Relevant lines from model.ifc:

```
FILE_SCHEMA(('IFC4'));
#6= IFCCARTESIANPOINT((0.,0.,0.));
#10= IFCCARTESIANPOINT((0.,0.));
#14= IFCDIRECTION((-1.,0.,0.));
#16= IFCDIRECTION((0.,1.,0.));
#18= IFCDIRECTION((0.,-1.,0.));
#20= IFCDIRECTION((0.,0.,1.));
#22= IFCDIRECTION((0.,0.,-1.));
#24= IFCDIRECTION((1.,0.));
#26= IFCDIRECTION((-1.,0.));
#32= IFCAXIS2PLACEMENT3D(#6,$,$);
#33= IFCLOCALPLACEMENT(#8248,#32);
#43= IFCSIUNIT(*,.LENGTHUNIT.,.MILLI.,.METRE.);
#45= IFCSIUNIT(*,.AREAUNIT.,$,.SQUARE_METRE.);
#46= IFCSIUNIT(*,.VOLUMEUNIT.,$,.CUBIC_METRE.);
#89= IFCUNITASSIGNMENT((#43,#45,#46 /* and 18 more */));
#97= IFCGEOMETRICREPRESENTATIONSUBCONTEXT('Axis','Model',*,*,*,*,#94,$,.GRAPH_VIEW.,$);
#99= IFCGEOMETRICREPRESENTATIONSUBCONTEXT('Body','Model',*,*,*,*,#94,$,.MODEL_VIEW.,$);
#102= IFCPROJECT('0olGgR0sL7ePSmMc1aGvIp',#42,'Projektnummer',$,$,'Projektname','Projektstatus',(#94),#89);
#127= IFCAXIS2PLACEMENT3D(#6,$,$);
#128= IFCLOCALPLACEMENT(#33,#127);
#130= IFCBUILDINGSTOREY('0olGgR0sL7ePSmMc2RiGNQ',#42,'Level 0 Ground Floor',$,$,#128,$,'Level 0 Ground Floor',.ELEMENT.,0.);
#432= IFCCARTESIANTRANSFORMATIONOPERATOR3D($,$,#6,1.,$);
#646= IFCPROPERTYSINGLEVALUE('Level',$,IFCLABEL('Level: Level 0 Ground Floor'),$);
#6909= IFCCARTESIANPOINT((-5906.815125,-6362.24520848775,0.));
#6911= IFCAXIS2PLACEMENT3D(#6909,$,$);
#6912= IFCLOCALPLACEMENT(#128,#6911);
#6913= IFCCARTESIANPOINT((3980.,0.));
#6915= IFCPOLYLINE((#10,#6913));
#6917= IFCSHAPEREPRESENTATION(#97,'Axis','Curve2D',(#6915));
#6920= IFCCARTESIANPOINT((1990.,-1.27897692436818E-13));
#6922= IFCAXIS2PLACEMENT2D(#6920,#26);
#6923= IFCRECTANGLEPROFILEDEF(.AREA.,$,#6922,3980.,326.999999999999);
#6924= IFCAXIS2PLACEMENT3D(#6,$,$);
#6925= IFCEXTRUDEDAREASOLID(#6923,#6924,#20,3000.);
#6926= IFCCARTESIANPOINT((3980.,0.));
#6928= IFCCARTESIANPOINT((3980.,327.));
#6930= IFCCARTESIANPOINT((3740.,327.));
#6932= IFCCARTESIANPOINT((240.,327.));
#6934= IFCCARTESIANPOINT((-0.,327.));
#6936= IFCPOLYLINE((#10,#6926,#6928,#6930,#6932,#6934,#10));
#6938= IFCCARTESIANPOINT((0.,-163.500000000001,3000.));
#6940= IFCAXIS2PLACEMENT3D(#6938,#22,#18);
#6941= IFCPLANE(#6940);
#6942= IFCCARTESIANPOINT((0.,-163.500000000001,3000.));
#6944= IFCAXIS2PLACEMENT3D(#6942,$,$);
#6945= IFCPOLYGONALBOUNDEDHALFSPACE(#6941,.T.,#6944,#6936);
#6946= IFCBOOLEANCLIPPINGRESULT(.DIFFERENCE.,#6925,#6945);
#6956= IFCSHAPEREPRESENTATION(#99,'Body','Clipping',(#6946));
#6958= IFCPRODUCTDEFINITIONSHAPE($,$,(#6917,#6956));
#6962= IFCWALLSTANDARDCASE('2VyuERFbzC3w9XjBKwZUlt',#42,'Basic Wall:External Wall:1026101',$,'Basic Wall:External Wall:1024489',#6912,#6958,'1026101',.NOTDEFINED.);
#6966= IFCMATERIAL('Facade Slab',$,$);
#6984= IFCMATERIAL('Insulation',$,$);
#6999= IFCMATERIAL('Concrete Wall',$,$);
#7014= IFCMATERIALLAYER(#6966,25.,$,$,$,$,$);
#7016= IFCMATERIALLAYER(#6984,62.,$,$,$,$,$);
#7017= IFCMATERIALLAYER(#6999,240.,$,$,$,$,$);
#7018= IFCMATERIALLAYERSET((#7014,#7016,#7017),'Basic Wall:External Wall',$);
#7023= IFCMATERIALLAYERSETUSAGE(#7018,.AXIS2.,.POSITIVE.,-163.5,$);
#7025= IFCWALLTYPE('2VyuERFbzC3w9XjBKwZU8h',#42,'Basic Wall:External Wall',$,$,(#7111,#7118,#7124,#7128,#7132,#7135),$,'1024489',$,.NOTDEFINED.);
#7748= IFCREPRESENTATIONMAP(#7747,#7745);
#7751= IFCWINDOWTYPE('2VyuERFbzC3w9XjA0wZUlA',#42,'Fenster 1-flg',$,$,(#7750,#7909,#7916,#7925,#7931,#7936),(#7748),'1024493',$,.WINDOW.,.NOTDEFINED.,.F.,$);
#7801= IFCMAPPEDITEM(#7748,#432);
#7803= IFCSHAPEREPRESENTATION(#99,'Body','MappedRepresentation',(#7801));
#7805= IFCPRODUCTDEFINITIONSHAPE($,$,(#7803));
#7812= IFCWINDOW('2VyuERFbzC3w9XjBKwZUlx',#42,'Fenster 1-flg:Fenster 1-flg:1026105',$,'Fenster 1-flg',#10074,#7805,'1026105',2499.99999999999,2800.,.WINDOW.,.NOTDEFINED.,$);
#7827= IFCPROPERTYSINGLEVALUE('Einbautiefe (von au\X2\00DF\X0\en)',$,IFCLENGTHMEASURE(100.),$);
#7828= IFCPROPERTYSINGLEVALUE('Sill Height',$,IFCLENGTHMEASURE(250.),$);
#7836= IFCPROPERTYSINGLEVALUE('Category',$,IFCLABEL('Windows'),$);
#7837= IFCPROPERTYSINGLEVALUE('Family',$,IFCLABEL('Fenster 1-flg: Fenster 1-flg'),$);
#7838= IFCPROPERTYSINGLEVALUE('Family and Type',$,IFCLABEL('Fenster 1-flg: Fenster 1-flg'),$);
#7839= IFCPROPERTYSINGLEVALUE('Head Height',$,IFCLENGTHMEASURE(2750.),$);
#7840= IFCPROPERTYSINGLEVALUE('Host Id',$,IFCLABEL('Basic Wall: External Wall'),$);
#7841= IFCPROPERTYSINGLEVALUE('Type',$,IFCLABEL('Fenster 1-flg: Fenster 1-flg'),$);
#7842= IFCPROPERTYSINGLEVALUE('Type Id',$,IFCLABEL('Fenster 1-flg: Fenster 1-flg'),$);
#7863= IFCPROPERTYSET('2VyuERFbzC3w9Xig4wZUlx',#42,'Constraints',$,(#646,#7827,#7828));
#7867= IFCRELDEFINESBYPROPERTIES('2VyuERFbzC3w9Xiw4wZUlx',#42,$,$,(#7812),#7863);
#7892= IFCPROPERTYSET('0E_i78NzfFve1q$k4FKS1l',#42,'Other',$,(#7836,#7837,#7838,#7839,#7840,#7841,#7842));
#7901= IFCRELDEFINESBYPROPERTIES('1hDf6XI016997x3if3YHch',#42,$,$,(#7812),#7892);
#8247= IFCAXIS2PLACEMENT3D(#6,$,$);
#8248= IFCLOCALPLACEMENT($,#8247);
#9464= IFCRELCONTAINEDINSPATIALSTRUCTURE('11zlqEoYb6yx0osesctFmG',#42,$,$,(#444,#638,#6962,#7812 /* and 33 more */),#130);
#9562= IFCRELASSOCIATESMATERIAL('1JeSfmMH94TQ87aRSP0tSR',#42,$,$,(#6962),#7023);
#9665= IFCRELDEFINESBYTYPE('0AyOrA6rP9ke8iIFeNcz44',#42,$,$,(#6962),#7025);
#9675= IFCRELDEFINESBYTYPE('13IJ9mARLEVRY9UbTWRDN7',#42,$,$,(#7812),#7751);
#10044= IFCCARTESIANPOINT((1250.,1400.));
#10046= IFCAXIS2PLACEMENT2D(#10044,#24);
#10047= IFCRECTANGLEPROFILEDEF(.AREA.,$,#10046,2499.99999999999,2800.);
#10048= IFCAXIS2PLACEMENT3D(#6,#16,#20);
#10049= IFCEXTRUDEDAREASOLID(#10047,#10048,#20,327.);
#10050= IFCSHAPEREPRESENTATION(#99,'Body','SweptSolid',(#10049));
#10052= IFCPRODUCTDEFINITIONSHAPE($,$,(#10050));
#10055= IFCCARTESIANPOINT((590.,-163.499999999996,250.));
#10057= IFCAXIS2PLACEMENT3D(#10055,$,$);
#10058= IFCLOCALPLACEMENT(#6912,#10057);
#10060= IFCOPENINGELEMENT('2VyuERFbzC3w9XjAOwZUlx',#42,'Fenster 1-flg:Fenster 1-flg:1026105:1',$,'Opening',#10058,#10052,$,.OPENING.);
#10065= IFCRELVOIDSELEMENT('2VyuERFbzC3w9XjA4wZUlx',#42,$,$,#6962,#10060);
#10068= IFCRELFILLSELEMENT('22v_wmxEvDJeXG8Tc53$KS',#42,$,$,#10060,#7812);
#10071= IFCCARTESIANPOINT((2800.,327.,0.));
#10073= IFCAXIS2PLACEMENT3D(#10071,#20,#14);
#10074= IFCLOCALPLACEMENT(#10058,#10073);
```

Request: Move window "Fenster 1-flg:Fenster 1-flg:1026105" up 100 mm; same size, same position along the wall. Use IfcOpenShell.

```python
import numpy as np
import ifcopenshell
import ifcopenshell.api.geometry
import ifcopenshell.api.pset
import ifcopenshell.util.element
import ifcopenshell.util.placement
import ifcopenshell.util.unit

model = ifcopenshell.open("model.ifc")
unit_scale = ifcopenshell.util.unit.calculate_unit_scale(model)

window = model.by_guid("2VyuERFbzC3w9XjBKwZUlx")
opening = window.FillsVoids[0].RelatingOpeningElement
dz = 100.0

shift = np.array([0.0, 0.0, dz])
# The window is placed relative to its opening, so it follows when the opening moves.
matrix = ifcopenshell.util.placement.get_local_placement(opening.ObjectPlacement)
matrix[:3, 3] += shift
ifcopenshell.api.geometry.edit_object_placement(
    model, product=opening, matrix=matrix, is_si=False, should_transform_children=True
)

# Keep the stored heights in step.
pset = model.by_id(ifcopenshell.util.element.get_pset(window, "Constraints", should_inherit=False)["id"])
ifcopenshell.api.pset.edit_pset(model, pset=pset, properties={
    "Sill Height": model.create_entity("IfcLengthMeasure", ifcopenshell.util.element.get_pset(window, "Constraints", "Sill Height") + dz),
})
pset = model.by_id(ifcopenshell.util.element.get_pset(window, "Other", should_inherit=False)["id"])
ifcopenshell.api.pset.edit_pset(model, pset=pset, properties={
    "Head Height": model.create_entity("IfcLengthMeasure", ifcopenshell.util.element.get_pset(window, "Other", "Head Height") + dz),
})

print(f"moved by {dz * unit_scale:+.3f} m")

model.write("model_rev.ifc")
```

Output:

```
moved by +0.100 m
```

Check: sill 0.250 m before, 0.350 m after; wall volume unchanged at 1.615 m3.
